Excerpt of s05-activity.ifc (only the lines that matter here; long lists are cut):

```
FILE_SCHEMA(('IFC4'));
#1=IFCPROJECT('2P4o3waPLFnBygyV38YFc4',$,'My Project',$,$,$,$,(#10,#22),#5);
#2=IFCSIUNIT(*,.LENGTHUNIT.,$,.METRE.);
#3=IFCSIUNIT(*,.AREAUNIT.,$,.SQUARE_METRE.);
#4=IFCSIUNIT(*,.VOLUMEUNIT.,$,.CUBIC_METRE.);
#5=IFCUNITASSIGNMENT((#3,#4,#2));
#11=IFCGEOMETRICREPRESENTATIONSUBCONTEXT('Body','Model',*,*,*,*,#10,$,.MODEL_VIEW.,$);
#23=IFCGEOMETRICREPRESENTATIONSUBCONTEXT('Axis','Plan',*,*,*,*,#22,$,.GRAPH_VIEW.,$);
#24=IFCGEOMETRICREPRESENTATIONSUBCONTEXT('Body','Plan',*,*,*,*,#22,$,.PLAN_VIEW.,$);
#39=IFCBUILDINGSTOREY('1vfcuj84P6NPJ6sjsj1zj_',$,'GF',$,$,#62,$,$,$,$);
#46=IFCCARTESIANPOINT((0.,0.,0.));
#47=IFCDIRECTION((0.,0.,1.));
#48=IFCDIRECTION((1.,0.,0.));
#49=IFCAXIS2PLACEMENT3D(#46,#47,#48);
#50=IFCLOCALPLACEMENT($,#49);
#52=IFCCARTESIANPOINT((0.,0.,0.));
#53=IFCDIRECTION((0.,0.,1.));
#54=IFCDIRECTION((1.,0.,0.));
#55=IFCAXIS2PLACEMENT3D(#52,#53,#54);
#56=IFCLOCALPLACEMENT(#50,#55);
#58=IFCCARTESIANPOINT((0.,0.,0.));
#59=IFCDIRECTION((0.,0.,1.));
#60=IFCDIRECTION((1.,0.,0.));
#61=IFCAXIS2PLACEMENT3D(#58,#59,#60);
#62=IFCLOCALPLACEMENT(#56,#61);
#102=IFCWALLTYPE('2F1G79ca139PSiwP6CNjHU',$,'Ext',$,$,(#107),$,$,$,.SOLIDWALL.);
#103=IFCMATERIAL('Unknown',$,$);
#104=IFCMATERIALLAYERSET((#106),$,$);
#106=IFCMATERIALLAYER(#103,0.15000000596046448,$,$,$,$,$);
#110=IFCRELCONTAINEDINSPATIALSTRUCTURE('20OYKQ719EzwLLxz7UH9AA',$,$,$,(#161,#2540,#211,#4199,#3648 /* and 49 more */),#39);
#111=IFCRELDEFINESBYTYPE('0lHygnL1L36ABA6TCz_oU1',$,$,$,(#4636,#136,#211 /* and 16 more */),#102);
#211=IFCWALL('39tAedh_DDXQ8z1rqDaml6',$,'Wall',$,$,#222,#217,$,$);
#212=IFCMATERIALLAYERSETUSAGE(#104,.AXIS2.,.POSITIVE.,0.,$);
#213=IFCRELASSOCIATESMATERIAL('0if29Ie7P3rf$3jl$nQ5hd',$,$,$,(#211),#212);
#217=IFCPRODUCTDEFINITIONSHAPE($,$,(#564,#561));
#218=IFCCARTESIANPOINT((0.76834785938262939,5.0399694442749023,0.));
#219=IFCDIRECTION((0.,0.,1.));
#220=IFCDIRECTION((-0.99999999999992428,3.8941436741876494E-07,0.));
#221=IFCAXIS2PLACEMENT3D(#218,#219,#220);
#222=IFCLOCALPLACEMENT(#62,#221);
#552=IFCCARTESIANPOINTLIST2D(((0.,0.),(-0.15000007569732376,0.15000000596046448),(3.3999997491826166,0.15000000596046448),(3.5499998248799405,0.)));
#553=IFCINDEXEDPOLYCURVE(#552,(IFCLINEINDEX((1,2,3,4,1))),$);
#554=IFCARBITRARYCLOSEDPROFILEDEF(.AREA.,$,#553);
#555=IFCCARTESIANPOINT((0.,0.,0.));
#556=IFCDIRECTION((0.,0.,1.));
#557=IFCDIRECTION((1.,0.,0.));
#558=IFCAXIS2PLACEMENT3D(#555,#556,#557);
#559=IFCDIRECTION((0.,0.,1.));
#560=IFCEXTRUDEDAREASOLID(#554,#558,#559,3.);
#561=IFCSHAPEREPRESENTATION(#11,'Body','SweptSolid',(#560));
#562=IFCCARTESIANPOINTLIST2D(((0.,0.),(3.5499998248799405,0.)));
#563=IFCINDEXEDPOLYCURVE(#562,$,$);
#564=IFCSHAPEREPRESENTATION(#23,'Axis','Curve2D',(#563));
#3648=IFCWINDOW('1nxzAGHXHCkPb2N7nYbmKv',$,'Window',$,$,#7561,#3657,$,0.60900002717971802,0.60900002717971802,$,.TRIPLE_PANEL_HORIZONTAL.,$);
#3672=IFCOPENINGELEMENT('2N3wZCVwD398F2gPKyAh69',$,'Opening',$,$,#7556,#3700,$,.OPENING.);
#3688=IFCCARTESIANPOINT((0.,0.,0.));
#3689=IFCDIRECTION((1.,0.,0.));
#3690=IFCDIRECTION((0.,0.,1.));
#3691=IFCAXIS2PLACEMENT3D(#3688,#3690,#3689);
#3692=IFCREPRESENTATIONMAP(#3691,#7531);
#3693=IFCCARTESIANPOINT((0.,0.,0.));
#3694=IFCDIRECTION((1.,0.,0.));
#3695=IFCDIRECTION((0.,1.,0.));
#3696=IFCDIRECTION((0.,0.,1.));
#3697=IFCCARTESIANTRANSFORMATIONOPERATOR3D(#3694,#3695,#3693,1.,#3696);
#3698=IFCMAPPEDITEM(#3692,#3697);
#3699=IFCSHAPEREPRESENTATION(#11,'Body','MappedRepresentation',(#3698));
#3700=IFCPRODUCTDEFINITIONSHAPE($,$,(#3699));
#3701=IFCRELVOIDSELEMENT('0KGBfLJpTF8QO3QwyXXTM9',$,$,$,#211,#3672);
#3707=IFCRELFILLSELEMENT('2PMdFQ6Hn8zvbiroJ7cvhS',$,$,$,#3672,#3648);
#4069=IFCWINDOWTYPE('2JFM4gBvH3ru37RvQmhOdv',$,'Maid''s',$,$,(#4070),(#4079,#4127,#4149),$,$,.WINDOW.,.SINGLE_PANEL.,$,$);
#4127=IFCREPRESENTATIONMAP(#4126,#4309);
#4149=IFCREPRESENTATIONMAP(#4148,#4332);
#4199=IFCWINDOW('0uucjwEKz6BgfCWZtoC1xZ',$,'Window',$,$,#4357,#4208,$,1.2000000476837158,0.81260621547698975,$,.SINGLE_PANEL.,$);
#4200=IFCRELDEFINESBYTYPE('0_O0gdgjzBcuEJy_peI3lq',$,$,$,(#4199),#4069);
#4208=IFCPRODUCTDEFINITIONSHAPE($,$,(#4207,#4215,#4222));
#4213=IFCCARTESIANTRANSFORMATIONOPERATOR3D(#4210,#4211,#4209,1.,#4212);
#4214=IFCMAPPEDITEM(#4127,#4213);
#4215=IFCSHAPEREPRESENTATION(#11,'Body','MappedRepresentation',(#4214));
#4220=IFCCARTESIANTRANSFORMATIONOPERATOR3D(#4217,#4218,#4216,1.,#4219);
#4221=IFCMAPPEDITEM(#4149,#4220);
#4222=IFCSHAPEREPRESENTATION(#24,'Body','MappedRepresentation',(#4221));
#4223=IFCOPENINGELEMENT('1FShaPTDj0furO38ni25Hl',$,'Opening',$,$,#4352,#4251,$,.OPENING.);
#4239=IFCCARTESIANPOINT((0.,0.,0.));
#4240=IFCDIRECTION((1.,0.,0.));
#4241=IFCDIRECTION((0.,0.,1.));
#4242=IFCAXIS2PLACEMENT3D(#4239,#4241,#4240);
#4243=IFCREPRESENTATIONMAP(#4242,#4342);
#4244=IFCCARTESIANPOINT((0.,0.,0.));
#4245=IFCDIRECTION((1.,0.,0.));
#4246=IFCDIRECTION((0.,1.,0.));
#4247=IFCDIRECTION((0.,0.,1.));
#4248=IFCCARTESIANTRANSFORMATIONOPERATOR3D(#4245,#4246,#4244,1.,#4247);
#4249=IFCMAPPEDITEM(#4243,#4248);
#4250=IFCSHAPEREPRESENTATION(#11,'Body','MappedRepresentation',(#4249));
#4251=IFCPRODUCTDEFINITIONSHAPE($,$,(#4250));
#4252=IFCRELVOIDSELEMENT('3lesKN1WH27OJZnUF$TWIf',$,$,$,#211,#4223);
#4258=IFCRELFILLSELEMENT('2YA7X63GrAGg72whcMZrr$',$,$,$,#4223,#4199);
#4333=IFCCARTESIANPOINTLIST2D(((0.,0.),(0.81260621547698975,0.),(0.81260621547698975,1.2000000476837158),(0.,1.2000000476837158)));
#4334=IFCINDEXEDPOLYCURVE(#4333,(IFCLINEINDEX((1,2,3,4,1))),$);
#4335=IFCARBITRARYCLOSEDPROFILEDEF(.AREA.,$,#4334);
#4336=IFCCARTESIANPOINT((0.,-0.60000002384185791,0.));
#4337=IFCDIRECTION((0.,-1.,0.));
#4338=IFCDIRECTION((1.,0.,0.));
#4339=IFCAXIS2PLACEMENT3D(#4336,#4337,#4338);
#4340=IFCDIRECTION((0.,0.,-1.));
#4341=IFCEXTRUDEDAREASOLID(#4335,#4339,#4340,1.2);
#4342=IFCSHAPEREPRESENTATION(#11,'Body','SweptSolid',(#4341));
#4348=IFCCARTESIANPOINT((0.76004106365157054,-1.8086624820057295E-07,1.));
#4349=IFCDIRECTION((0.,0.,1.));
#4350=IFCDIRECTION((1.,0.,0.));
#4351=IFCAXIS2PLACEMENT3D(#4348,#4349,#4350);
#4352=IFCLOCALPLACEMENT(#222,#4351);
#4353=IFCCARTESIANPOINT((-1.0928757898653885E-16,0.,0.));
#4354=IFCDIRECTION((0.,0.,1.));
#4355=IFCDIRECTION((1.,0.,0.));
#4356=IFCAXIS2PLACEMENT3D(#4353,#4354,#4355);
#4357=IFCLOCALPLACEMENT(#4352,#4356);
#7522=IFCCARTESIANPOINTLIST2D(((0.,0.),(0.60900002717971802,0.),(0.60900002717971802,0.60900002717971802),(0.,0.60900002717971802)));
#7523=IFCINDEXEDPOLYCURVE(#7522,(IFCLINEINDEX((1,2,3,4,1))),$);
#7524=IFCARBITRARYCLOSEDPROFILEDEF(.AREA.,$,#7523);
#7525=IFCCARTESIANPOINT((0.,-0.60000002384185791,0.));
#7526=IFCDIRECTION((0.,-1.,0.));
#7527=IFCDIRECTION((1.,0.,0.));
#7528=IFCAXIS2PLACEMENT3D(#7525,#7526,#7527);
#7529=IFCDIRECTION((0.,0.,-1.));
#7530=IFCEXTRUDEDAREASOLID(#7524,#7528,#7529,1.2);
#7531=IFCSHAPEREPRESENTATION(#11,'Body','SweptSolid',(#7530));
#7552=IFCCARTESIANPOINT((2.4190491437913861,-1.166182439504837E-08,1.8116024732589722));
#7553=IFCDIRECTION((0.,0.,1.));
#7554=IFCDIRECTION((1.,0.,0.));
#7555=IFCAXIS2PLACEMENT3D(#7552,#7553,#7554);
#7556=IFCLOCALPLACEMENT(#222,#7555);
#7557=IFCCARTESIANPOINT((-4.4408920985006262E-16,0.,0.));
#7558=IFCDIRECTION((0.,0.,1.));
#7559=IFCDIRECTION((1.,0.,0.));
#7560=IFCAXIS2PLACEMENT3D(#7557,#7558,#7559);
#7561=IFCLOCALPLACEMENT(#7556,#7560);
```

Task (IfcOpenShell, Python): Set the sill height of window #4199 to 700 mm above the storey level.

```python
import numpy as np
import ifcopenshell
import ifcopenshell.api.geometry
import ifcopenshell.geom
import ifcopenshell.util.element
import ifcopenshell.util.placement
import ifcopenshell.util.shape
import ifcopenshell.util.unit

model = ifcopenshell.open("s05-activity.ifc")
unit_scale = ifcopenshell.util.unit.calculate_unit_scale(model)

window = model.by_guid("0uucjwEKz6BgfCWZtoC1xZ")
opening = window.FillsVoids[0].RelatingOpeningElement
storey = ifcopenshell.util.element.get_container(window, ifc_class="IfcBuildingStorey")
level = ifcopenshell.util.placement.get_local_placement(storey.ObjectPlacement)[2, 3]

# The opening's origin need not be at the sill, so measure its lowest point.
shape = ifcopenshell.geom.create_shape(ifcopenshell.geom.settings(), opening)
bottom = ifcopenshell.util.shape.get_shape_bottom_elevation(shape, shape.geometry) / unit_scale
dz = level + 0.7 - bottom

shift = np.array([0.0, 0.0, dz])
# The window is placed relative to its opening, so it follows when the opening moves.
matrix = ifcopenshell.util.placement.get_local_placement(opening.ObjectPlacement)
matrix[:3, 3] += shift
ifcopenshell.api.geometry.edit_object_placement(
    model, product=opening, matrix=matrix, is_si=False, should_transform_children=True
)

print(f"moved by {dz * unit_scale:+.3f} m")

model.write("s05-activity_edited.ifc")
```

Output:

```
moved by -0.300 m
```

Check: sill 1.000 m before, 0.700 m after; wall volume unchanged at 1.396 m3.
